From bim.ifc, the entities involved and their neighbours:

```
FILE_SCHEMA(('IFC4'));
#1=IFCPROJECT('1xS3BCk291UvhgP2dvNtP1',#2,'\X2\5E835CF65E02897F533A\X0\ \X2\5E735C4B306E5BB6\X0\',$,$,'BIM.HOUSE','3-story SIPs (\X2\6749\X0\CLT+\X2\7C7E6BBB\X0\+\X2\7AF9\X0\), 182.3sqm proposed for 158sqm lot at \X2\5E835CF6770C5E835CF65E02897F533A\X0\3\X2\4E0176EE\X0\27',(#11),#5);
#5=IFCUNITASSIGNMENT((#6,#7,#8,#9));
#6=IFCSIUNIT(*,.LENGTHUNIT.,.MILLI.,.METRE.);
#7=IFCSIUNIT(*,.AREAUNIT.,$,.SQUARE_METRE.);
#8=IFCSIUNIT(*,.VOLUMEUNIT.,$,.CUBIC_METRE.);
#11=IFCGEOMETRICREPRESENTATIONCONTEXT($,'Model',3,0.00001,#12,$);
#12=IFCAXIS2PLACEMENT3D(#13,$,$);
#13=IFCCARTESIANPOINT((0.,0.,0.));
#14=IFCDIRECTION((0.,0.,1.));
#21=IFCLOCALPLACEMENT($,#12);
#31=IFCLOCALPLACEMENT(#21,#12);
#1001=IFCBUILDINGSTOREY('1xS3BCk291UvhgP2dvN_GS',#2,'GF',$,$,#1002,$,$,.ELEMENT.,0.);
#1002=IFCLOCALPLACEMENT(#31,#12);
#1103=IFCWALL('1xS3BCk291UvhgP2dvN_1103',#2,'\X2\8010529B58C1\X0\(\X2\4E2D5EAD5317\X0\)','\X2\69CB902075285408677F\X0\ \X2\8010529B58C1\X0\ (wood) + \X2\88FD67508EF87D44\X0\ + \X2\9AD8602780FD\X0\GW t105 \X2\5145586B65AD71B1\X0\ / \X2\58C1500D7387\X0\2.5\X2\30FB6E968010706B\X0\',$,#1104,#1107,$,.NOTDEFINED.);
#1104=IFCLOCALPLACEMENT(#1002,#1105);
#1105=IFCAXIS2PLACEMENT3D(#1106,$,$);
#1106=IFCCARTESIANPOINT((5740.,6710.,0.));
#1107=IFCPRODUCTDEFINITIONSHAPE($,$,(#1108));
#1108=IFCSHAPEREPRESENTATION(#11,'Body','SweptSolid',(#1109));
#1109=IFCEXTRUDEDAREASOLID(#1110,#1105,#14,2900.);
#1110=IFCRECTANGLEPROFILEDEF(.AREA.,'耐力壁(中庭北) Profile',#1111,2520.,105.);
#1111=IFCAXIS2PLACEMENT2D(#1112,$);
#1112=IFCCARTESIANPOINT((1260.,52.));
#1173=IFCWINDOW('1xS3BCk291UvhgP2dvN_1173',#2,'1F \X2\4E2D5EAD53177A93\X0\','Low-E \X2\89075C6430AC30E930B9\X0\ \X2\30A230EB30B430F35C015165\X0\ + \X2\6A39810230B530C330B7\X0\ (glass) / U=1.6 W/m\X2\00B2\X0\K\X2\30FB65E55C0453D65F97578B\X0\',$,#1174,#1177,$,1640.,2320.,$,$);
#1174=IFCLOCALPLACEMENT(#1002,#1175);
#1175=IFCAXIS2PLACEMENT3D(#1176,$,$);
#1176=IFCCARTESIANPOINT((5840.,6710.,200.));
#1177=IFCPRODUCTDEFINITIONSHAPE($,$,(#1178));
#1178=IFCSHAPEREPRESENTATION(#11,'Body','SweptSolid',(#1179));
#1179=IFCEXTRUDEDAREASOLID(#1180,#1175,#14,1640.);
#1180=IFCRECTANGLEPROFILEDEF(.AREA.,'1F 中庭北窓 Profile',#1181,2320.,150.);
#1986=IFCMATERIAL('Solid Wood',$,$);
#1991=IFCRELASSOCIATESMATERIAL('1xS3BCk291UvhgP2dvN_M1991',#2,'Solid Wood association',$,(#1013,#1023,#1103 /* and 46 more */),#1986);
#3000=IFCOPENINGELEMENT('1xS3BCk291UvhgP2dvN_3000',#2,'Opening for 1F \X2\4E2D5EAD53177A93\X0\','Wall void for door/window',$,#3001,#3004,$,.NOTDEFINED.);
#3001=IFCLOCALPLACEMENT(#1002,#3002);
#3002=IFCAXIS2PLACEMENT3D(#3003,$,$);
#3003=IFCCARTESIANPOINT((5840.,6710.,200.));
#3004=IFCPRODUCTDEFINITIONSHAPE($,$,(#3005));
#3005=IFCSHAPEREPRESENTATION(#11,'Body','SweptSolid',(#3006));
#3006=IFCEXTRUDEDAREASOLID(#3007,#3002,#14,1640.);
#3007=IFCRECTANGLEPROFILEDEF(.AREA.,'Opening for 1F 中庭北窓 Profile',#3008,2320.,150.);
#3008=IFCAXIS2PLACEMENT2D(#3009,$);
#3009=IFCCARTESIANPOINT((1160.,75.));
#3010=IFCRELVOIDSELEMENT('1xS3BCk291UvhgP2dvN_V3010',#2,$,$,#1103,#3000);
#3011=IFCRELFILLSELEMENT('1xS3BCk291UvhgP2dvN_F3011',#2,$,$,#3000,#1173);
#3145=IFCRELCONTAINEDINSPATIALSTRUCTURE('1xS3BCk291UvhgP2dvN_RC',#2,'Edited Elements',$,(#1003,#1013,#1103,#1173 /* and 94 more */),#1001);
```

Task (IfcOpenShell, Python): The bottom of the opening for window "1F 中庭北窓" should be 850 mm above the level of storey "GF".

```python
import numpy as np
import ifcopenshell
import ifcopenshell.api.geometry
import ifcopenshell.geom
import ifcopenshell.util.element
import ifcopenshell.util.placement
import ifcopenshell.util.shape
import ifcopenshell.util.unit

model = ifcopenshell.open("bim.ifc")
unit_scale = ifcopenshell.util.unit.calculate_unit_scale(model)

window = model.by_guid("1xS3BCk291UvhgP2dvN_1173")
opening = window.FillsVoids[0].RelatingOpeningElement
storey = ifcopenshell.util.element.get_container(window, ifc_class="IfcBuildingStorey")
level = ifcopenshell.util.placement.get_local_placement(storey.ObjectPlacement)[2, 3]

# The opening's origin need not be at the sill, so measure its lowest point.
shape = ifcopenshell.geom.create_shape(ifcopenshell.geom.settings(), opening)
bottom = ifcopenshell.util.shape.get_shape_bottom_elevation(shape, shape.geometry) / unit_scale
dz = level + 850.0 - bottom

shift = np.array([0.0, 0.0, dz])
# The window is not placed relative to its opening, so move both.
for product in (opening, window):
    matrix = ifcopenshell.util.placement.get_local_placement(product.ObjectPlacement)
    matrix[:3, 3] += shift
    ifcopenshell.api.geometry.edit_object_placement(model, product=product, matrix=matrix, is_si=False)

print(f"moved by {dz * unit_scale:+.3f} m")

model.write("bim_edited.ifc")
```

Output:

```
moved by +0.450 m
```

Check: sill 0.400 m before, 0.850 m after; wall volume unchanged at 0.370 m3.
